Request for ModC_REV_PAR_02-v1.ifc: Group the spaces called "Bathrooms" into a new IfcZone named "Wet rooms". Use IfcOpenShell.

First a look at what the model holds.

```python
import ifcopenshell

model = ifcopenshell.open("ModC_REV_PAR_02-v1.ifc")
print(model.schema)
seen = {}
for space in model.by_type("IfcSpace"):
    seen[space.LongName] = seen.get(space.LongName, 0) + 1
for name, count in sorted(seen.items(), key=str):
    print(count, "x", name)
print("zones:", [z.Name for z in model.by_type("IfcZone")][:20])
```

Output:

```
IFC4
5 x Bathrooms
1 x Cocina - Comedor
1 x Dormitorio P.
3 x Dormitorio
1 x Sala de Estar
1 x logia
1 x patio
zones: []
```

```python
import ifcopenshell
import ifcopenshell.api.group
import ifcopenshell.api.root

model = ifcopenshell.open("ModC_REV_PAR_02-v1.ifc")

names = {"Bathrooms"}
spaces = [s for s in model.by_type("IfcSpace") if s.LongName in names]

zone = ifcopenshell.api.root.create_entity(model, ifc_class="IfcZone", name="Wet rooms")
ifcopenshell.api.group.assign_group(model, products=spaces, group=zone)
print(len(spaces), "spaces in", zone.Name)

model.write("ModC_REV_PAR_02-v1_v2.ifc")
```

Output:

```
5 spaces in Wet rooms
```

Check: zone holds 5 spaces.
